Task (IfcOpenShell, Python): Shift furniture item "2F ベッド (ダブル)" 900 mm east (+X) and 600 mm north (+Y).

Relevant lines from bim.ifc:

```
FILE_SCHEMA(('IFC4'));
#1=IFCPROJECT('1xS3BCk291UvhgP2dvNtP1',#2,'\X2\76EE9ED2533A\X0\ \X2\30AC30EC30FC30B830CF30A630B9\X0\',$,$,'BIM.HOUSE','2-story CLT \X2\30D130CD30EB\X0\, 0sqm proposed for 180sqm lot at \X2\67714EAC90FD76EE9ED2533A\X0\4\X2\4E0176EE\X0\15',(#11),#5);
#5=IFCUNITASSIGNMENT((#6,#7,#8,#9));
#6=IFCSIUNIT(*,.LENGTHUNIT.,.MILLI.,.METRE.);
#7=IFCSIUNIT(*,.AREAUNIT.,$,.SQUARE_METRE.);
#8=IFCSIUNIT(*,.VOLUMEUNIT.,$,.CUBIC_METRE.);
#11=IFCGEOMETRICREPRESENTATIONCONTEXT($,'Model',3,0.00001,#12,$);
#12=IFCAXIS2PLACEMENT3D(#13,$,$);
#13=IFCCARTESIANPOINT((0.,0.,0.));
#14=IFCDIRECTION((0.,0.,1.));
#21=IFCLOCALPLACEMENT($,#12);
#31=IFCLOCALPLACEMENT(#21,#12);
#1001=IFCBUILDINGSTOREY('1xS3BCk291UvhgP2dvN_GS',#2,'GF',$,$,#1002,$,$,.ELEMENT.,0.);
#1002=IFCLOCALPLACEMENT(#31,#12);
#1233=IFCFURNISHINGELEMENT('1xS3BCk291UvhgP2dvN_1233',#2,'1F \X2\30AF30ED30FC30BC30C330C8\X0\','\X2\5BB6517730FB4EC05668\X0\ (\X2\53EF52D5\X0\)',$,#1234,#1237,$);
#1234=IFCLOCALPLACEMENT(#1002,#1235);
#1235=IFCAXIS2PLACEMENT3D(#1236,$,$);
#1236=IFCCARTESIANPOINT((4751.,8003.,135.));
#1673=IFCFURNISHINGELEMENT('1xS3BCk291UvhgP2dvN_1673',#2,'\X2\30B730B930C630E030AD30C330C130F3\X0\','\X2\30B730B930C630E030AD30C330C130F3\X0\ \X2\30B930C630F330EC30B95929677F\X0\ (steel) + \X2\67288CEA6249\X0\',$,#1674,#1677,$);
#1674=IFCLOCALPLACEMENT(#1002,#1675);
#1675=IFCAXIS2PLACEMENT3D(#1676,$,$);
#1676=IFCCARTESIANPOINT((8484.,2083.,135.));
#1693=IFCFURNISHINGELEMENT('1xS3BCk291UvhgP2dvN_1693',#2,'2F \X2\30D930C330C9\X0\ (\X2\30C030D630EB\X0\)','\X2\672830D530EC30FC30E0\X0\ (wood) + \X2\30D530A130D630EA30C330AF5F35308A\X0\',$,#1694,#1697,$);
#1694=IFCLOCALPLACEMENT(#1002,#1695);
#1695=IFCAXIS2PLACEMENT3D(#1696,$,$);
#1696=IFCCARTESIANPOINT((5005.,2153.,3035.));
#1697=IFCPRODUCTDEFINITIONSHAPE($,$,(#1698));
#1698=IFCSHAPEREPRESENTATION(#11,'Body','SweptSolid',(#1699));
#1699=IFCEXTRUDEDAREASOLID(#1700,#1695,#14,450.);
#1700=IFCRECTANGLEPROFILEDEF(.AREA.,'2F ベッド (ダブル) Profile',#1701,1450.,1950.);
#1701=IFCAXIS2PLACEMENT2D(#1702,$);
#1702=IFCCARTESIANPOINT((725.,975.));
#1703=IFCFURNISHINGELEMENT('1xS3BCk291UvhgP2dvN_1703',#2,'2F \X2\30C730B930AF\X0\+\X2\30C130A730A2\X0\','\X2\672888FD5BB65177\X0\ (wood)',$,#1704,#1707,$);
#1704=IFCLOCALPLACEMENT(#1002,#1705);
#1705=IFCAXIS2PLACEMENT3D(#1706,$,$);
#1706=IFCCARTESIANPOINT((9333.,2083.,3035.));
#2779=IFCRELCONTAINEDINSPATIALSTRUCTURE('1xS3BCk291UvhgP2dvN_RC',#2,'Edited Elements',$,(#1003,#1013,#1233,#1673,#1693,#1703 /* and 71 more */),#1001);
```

```python
import ifcopenshell
import ifcopenshell.api.geometry
import ifcopenshell.util.placement
import ifcopenshell.util.unit

model = ifcopenshell.open("bim.ifc")
unit_scale = ifcopenshell.util.unit.calculate_unit_scale(model)

item = model.by_guid("1xS3BCk291UvhgP2dvN_1693")
matrix = ifcopenshell.util.placement.get_local_placement(item.ObjectPlacement)
matrix[0, 3] += 0.9 / unit_scale
matrix[1, 3] += 0.6 / unit_scale
ifcopenshell.api.geometry.edit_object_placement(model, product=item, matrix=matrix, is_si=False)

print(ifcopenshell.util.placement.get_local_placement(item.ObjectPlacement).round(3) + 0.0)

model.write("bim-out.ifc")
```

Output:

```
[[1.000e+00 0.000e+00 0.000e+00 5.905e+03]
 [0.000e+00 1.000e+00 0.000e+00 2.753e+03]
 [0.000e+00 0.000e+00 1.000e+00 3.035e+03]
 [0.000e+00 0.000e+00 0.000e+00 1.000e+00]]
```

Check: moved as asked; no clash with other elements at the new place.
